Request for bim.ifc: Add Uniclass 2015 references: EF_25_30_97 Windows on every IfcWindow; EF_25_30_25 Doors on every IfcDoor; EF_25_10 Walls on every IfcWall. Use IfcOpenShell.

First a look at what the model holds.

```python
import ifcopenshell

model = ifcopenshell.open("bim.ifc")
print(model.schema)
print("classifications:", [c.Name for c in model.by_type("IfcClassification")])
for ifc_class in ("IfcDoor", "IfcRoof", "IfcStair", "IfcWall", "IfcWindow"):
    print(ifc_class, len(model.by_type(ifc_class)))
```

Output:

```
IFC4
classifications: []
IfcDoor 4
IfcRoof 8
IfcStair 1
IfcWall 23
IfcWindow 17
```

```python
import ifcopenshell
import ifcopenshell.api.classification

model = ifcopenshell.open("bim.ifc")

system = ifcopenshell.api.classification.add_classification(model, classification="Uniclass 2015")

codes = {
    "IfcWindow": ("EF_25_30_97", "Windows"),
    "IfcDoor": ("EF_25_30_25", "Doors"),
    "IfcWall": ("EF_25_10", "Walls"),
}
for ifc_class, (code, name) in codes.items():
    products = model.by_type(ifc_class)
    ifcopenshell.api.classification.add_reference(
        model, products=products, classification=system, identification=code, name=name
    )
    print(code, len(products))

model.write("bim_rev.ifc")
```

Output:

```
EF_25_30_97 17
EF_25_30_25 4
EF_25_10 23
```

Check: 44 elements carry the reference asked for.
